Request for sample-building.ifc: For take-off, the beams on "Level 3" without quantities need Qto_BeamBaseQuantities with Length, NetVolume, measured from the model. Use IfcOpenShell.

First a look at what the model holds.

```python
import ifcopenshell
import ifcopenshell.util.element
import ifcopenshell.util.unit

model = ifcopenshell.open("sample-building.ifc")
print(model.schema)
for unit_type in ("LENGTHUNIT", "AREAUNIT", "VOLUMEUNIT"):
    print(unit_type, ifcopenshell.util.unit.calculate_unit_scale(model, unit_type))
storey = next(s for s in model.by_type("IfcBuildingStorey") if s.Name == "Level 3")
beams = [e for e in ifcopenshell.util.element.get_decomposition(storey) if e.is_a("IfcBeam")]
for e in sorted(beams, key=lambda e: e.id()):
    print(e.id(), e.is_a(), e.Name, list(ifcopenshell.util.element.get_psets(e, qtos_only=True)), sep=" | ")
```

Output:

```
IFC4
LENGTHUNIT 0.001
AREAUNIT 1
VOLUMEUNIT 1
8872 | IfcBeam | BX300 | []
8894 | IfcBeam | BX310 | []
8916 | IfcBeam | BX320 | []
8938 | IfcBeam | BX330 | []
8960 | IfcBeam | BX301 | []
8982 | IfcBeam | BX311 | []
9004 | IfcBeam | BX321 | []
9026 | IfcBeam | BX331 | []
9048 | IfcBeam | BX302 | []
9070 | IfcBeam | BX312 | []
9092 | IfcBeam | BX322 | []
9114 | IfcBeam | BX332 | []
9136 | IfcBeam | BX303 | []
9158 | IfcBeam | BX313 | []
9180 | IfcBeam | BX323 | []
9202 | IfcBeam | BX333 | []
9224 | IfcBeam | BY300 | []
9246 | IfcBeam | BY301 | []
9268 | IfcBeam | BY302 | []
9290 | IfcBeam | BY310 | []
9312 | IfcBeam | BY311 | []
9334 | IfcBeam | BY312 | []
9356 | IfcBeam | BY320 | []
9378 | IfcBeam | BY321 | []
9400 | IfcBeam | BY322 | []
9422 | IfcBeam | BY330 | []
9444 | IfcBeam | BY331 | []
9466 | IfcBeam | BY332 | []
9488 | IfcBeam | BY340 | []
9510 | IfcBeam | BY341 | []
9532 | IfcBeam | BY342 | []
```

```python
import ifcopenshell
import ifcopenshell.api.pset
import ifcopenshell.geom
import ifcopenshell.util.element
import ifcopenshell.util.shape
import ifcopenshell.util.unit

model = ifcopenshell.open("sample-building.ifc")
unit_scale = ifcopenshell.util.unit.calculate_unit_scale(model)
volume_scale = ifcopenshell.util.unit.calculate_unit_scale(model, "VOLUMEUNIT")
settings = ifcopenshell.geom.settings()

storey = next(s for s in model.by_type("IfcBuildingStorey") if s.Name == "Level 3")
beams = [e for e in ifcopenshell.util.element.get_decomposition(storey) if e.is_a("IfcBeam")]

for e in sorted(beams, key=lambda e: e.id()):
    if ifcopenshell.util.element.get_psets(e, qtos_only=True, should_inherit=False):
        continue
    # Geometry comes back in metres, in the element's own axes.
    shape = ifcopenshell.geom.create_shape(settings, e)
    values = {
        "Length": ifcopenshell.util.shape.get_max_xyz(shape.geometry) / unit_scale,
        "NetVolume": ifcopenshell.util.shape.get_volume(shape.geometry) / volume_scale,
    }
    qto = ifcopenshell.api.pset.add_qto(model, product=e, name="Qto_BeamBaseQuantities")
    ifcopenshell.api.pset.edit_qto(model, qto=qto, properties=values)
    print(e.id(), {k: round(v, 3) for k, v in values.items()})

model.write("sample-building_v2.ifc")
```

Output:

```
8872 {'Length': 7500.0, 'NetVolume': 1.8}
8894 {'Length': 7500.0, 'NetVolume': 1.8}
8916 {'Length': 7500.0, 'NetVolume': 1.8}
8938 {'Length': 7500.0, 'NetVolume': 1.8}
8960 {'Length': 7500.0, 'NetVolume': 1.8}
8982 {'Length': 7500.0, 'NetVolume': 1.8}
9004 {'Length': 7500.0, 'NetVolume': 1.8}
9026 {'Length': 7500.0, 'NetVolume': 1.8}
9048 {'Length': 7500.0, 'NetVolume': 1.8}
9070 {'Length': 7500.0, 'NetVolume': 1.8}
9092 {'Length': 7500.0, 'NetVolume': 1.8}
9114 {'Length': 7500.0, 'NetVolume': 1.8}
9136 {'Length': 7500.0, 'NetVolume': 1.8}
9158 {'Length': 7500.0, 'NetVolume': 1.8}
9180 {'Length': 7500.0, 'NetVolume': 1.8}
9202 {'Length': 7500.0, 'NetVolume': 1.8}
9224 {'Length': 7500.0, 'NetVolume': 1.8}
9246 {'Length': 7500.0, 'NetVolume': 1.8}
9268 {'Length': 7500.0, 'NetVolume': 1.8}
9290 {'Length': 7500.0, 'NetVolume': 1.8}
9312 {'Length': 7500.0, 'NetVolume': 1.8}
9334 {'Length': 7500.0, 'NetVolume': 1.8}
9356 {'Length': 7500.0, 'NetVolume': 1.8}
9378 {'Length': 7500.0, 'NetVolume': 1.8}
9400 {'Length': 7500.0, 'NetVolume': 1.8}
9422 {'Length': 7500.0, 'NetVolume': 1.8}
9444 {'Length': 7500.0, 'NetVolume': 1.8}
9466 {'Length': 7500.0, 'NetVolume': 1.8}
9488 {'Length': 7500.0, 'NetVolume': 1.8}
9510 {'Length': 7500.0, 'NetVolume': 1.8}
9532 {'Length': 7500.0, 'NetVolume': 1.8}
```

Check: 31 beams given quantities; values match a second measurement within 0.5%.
